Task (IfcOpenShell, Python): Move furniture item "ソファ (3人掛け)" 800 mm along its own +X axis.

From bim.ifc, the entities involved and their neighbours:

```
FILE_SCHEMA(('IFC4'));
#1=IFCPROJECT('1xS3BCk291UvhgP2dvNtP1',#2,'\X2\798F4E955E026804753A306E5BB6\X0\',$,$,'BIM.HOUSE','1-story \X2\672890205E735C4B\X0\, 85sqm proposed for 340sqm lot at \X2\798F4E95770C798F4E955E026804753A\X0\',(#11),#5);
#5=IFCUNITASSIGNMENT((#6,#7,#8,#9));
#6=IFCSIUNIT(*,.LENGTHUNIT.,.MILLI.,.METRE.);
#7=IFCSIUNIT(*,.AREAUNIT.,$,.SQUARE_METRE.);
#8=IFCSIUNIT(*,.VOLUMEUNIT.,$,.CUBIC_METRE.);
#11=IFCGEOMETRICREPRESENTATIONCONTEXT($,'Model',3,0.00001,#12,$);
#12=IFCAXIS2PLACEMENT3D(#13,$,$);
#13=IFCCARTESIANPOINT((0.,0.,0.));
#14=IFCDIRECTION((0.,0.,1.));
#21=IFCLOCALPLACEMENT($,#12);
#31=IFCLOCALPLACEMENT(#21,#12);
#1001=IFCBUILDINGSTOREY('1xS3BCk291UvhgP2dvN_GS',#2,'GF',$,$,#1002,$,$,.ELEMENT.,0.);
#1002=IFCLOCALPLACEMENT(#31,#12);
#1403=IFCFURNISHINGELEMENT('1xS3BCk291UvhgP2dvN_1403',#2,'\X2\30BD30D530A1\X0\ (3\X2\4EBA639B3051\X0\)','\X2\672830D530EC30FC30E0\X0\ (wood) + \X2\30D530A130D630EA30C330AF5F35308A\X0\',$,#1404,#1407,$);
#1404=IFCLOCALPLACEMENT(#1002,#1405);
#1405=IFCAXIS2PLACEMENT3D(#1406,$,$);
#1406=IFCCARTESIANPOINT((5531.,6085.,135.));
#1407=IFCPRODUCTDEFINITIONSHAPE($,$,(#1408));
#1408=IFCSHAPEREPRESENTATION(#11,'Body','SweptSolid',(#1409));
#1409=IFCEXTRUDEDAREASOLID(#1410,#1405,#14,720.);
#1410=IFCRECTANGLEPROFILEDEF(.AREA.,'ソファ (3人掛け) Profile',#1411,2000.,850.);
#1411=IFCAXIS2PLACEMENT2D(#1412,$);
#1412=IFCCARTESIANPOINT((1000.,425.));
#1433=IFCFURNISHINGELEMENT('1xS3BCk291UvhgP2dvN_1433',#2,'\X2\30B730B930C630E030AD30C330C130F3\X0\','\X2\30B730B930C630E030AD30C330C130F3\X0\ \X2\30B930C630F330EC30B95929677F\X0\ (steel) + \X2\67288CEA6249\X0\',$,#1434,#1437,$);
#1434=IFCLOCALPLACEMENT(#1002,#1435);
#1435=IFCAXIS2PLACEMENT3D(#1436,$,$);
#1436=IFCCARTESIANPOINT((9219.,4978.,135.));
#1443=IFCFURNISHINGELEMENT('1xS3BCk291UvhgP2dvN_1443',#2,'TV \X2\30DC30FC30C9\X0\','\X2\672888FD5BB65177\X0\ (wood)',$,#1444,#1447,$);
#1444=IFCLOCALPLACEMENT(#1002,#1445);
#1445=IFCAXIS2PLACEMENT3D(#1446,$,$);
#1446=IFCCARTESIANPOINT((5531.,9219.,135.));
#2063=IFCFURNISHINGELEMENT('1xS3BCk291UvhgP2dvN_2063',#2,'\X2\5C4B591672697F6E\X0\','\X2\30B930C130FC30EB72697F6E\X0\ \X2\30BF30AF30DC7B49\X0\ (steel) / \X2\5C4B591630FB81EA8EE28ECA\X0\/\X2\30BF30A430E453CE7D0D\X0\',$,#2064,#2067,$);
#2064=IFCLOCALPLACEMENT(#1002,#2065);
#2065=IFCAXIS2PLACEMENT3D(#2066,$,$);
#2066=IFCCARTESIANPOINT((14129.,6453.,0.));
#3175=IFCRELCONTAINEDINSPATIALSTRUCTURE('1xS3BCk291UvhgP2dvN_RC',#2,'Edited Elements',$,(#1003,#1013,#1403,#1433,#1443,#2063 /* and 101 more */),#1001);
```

```python
import ifcopenshell
import ifcopenshell.api.geometry
import ifcopenshell.util.placement

model = ifcopenshell.open("bim.ifc")

item = model.by_id(1403)
matrix = ifcopenshell.util.placement.get_local_placement(item.ObjectPlacement)
matrix[:3, 3] += matrix[:3, 0] * 800.0
ifcopenshell.api.geometry.edit_object_placement(model, product=item, matrix=matrix, is_si=False)

print(ifcopenshell.util.placement.get_local_placement(item.ObjectPlacement).round(3) + 0.0)

model.write("bim_rev.ifc")
```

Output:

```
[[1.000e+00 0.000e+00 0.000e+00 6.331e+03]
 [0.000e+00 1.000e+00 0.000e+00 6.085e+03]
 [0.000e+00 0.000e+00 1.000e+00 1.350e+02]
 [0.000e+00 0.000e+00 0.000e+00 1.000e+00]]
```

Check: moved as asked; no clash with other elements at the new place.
